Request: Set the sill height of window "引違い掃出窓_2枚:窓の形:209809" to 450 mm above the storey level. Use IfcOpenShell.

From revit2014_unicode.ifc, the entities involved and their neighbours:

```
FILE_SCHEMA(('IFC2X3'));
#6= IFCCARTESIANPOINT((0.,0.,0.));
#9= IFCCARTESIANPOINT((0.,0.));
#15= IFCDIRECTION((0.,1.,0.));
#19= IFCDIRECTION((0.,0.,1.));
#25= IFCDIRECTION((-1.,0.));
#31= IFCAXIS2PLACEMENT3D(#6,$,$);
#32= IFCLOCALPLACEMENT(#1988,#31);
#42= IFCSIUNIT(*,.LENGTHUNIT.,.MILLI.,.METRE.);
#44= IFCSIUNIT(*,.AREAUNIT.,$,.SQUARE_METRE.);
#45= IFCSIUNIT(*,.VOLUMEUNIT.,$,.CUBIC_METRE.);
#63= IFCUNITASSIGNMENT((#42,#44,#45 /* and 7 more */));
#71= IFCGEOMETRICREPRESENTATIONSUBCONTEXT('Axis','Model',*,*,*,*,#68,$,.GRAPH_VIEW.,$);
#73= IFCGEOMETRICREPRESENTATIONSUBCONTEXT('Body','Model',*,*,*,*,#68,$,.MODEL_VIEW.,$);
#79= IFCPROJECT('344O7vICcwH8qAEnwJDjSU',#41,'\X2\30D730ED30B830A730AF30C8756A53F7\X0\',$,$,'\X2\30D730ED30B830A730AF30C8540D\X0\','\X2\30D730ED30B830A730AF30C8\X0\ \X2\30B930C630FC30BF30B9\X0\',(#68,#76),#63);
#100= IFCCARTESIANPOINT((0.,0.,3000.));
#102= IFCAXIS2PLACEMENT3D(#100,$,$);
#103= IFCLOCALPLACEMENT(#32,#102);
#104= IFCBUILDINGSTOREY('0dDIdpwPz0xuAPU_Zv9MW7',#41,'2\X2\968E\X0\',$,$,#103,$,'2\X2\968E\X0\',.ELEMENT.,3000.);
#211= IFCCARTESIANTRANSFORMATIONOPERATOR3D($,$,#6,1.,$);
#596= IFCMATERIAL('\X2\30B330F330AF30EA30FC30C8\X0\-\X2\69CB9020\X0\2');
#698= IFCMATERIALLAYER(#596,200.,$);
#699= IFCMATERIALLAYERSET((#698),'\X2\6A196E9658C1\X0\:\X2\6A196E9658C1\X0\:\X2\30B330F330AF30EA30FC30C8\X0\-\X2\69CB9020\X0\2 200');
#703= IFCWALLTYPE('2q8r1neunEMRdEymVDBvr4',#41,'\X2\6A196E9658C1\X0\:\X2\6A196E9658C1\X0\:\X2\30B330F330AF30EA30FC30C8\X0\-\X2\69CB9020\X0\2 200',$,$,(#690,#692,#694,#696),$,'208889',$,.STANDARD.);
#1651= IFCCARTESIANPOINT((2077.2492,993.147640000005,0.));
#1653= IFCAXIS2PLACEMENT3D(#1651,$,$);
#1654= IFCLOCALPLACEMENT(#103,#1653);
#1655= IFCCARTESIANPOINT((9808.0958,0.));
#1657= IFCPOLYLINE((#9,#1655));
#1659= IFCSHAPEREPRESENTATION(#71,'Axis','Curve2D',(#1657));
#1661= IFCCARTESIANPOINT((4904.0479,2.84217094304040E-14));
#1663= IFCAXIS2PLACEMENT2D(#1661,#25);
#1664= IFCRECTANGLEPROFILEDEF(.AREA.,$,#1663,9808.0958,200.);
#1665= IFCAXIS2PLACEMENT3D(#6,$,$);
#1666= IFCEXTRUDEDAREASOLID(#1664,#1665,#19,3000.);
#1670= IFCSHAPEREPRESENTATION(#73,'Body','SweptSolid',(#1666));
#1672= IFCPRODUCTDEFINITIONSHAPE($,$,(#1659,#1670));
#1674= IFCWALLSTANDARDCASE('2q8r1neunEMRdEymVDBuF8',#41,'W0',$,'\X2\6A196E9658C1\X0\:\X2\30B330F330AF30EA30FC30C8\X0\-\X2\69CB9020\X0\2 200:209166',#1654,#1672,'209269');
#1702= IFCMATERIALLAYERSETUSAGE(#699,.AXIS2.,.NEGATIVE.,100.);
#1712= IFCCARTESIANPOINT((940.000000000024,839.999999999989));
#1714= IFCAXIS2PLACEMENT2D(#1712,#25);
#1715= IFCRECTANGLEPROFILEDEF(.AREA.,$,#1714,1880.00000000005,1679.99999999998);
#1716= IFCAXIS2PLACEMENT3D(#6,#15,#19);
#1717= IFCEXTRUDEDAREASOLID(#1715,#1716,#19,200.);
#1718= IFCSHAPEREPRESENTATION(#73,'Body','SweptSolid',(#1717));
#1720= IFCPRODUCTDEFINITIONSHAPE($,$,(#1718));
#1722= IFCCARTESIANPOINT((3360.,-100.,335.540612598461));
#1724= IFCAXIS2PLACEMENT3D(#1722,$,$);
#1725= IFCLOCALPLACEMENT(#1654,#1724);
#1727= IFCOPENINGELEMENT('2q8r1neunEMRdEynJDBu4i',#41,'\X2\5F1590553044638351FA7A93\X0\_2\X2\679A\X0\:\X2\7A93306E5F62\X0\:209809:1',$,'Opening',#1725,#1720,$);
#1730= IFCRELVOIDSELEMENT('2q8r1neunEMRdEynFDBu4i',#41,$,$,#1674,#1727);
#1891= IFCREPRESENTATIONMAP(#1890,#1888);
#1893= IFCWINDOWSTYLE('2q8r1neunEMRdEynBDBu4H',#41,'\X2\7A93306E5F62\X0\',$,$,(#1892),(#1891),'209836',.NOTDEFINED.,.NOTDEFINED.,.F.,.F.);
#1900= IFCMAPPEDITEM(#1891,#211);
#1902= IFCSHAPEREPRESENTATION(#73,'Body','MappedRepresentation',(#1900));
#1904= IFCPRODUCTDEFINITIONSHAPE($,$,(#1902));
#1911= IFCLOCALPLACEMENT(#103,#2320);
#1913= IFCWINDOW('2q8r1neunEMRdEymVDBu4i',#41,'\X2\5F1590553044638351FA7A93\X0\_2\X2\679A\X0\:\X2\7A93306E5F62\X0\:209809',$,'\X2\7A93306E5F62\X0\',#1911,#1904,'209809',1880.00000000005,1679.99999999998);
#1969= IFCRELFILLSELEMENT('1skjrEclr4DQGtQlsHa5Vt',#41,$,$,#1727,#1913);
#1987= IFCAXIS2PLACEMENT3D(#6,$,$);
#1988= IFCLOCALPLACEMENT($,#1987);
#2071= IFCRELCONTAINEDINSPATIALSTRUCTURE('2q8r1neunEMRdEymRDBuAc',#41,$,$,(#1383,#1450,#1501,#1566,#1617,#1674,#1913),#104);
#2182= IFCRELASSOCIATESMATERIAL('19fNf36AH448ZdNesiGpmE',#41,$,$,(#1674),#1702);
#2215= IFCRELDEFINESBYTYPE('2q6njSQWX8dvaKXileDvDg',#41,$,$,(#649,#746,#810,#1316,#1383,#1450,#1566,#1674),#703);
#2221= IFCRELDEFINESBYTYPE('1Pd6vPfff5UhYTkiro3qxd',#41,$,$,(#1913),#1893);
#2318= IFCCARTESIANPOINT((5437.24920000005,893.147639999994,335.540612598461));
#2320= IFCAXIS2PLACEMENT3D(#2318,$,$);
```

```python
import numpy as np
import ifcopenshell
import ifcopenshell.api.geometry
import ifcopenshell.geom
import ifcopenshell.util.element
import ifcopenshell.util.placement
import ifcopenshell.util.shape
import ifcopenshell.util.unit

model = ifcopenshell.open("revit2014_unicode.ifc")
unit_scale = ifcopenshell.util.unit.calculate_unit_scale(model)

window = model.by_guid("2q8r1neunEMRdEymVDBu4i")
opening = window.FillsVoids[0].RelatingOpeningElement
storey = ifcopenshell.util.element.get_container(window, ifc_class="IfcBuildingStorey")
level = ifcopenshell.util.placement.get_local_placement(storey.ObjectPlacement)[2, 3]

# The opening's origin need not be at the sill, so measure its lowest point.
shape = ifcopenshell.geom.create_shape(ifcopenshell.geom.settings(), opening)
bottom = ifcopenshell.util.shape.get_shape_bottom_elevation(shape, shape.geometry) / unit_scale
dz = level + 450.0 - bottom

shift = np.array([0.0, 0.0, dz])
# The window is not placed relative to its opening, so move both.
for product in (opening, window):
    matrix = ifcopenshell.util.placement.get_local_placement(product.ObjectPlacement)
    matrix[:3, 3] += shift
    ifcopenshell.api.geometry.edit_object_placement(model, product=product, matrix=matrix, is_si=False)

print(f"moved by {dz * unit_scale:+.3f} m")

model.write("revit2014_unicode_updated.ifc")
```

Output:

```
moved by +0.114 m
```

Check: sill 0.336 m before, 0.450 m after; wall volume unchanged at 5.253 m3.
